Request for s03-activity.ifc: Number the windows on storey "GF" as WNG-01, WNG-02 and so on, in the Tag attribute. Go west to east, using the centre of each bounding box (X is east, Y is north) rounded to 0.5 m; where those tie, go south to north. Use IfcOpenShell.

First a look at what the model holds.

```python
import ifcopenshell
import ifcopenshell.util.element
import ifcopenshell.util.placement

model = ifcopenshell.open("s03-activity.ifc")
print(model.schema)
storey = next(s for s in model.by_type("IfcBuildingStorey") if s.Name == "GF")
windows = [e for e in ifcopenshell.util.element.get_decomposition(storey) if e.is_a("IfcWindow")]
for e in sorted(windows, key=lambda e: e.id()):
    origin = ifcopenshell.util.placement.get_local_placement(e.ObjectPlacement)[:3, 3]
    print(e.id(), e.Tag, e.Name, origin.round(2) + 0.0, sep=" | ")
```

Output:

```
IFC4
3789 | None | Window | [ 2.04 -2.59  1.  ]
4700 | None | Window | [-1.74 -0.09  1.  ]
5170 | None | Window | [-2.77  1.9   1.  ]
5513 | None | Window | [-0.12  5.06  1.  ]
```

```python
import ifcopenshell
import ifcopenshell.geom
import ifcopenshell.util.element
import ifcopenshell.util.shape

model = ifcopenshell.open("s03-activity.ifc")
settings = ifcopenshell.geom.settings()
settings.set("use-world-coords", True)


def centre(element):
    shape = ifcopenshell.geom.create_shape(settings, element)
    return ifcopenshell.util.shape.get_bbox_centroid(shape.geometry)


storey = next(s for s in model.by_type("IfcBuildingStorey") if s.Name == "GF")
windows = [e for e in ifcopenshell.util.element.get_decomposition(storey) if e.is_a("IfcWindow")]

# Insertion points can sit at a corner or the storey origin, so sort by the geometry (in metres).
centres = {e: centre(e) for e in windows}
windows.sort(key=lambda e: (round(centres[e][0] / 0.5), centres[e][1]))

for i, e in enumerate(windows, start=1):
    number = f"WNG-{i:02d}"
    e.Tag = number
    print(e.id(), number)

model.write("s03-activity_updated.ifc")
```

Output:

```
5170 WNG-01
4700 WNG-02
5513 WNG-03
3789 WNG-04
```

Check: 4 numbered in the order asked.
